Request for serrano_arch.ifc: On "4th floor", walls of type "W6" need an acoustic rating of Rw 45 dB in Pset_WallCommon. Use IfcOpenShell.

First a look at what the model holds.

```python
import ifcopenshell
import ifcopenshell.util.element

model = ifcopenshell.open("serrano_arch.ifc")
print(model.schema)
storey = next(s for s in model.by_type("IfcBuildingStorey") if s.Name == "4th floor")
walls = [e for e in ifcopenshell.util.element.get_decomposition(storey) if e.is_a("IfcWall")]
seen = {}
for e in walls:
    element_type = ifcopenshell.util.element.get_type(e)
    key = (element_type.Name if element_type != e and element_type else None, ifcopenshell.util.element.get_pset(e, "Pset_WallCommon", "AcousticRating"))
    seen[key] = seen.get(key, 0) + 1
for (name, value), count in sorted(seen.items(), key=str):
    print(count, "x", name, "|", value)
```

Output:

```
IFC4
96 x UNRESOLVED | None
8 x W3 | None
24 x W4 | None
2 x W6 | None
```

```python
import ifcopenshell
import ifcopenshell.api.pset
import ifcopenshell.util.element

model = ifcopenshell.open("serrano_arch.ifc")

storey = next(s for s in model.by_type("IfcBuildingStorey") if s.Name == "4th floor")
walls = [e for e in ifcopenshell.util.element.get_decomposition(storey) if e.is_a("IfcWall")]

count = 0
for e in walls:
    element_type = ifcopenshell.util.element.get_type(e)
    if element_type in (None, e) or element_type.Name != "W6":
        continue
    # add_pset returns the element's existing set when there is one.
    pset = ifcopenshell.api.pset.add_pset(model, product=e, name="Pset_WallCommon")
    ifcopenshell.api.pset.edit_pset(model, pset=pset, properties={"AcousticRating": "Rw 45 dB"})
    count += 1

print(count, "walls updated")

model.write("serrano_arch_updated.ifc")
```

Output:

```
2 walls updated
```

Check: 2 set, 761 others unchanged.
